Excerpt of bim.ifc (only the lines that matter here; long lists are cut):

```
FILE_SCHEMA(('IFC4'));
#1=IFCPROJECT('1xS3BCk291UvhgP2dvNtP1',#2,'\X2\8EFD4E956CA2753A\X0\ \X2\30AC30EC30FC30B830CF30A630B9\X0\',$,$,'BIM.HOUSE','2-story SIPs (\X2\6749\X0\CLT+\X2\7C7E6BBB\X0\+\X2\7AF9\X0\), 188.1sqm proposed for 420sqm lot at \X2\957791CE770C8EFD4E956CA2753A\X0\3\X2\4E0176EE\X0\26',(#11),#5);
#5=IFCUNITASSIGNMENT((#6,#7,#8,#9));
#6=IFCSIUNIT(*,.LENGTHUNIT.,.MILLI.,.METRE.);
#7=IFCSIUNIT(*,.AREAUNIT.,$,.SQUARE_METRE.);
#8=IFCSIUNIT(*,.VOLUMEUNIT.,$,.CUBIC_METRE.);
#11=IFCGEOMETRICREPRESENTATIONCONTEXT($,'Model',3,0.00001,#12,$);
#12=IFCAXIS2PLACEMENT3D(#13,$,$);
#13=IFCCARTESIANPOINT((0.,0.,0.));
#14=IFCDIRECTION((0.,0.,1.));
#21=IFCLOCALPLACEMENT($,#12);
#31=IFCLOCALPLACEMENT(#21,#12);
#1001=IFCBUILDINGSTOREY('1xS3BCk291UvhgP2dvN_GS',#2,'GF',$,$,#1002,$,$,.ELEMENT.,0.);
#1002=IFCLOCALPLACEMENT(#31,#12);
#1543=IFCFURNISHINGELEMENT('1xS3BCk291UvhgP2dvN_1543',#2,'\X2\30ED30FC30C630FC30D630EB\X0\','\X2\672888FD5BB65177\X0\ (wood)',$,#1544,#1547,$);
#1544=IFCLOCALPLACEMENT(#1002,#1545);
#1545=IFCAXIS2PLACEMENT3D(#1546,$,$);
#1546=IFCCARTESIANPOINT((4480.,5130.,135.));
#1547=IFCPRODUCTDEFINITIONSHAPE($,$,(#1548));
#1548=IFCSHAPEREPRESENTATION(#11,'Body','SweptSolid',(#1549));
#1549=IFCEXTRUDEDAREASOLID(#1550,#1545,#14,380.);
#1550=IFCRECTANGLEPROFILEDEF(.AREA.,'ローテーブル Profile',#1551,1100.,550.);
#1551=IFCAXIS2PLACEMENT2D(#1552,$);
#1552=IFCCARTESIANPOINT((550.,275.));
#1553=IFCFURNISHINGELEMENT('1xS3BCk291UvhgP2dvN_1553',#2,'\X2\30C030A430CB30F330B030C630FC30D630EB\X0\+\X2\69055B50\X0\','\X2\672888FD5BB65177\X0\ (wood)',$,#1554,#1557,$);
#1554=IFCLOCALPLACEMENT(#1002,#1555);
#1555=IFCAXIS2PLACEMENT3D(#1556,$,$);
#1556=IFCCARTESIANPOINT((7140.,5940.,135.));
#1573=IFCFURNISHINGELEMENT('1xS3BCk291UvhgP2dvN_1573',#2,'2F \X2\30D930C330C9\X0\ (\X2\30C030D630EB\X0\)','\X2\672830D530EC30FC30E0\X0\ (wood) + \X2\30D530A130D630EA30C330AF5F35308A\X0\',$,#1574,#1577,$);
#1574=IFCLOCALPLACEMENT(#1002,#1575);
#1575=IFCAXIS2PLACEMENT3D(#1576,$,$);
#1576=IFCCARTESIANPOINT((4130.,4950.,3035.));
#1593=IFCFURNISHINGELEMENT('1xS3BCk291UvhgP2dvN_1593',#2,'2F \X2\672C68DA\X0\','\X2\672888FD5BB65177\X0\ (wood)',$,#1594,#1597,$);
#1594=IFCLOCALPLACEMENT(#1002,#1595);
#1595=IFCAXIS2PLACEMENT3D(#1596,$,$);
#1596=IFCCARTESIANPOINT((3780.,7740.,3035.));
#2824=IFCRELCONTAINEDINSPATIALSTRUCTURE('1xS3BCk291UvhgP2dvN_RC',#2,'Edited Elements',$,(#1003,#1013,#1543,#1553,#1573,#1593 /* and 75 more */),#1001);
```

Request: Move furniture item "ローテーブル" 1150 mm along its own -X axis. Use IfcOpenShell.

```python
import ifcopenshell
import ifcopenshell.api.geometry
import ifcopenshell.util.placement

model = ifcopenshell.open("bim.ifc")

item = model.by_guid("1xS3BCk291UvhgP2dvN_1543")
matrix = ifcopenshell.util.placement.get_local_placement(item.ObjectPlacement)
matrix[:3, 3] -= matrix[:3, 0] * 1150.0
ifcopenshell.api.geometry.edit_object_placement(model, product=item, matrix=matrix, is_si=False)

print(ifcopenshell.util.placement.get_local_placement(item.ObjectPlacement).round(3) + 0.0)

model.write("bim_updated.ifc")
```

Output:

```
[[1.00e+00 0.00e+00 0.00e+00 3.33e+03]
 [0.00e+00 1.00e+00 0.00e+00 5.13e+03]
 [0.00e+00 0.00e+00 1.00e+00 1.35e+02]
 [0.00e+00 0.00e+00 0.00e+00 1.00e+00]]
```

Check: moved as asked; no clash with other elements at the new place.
